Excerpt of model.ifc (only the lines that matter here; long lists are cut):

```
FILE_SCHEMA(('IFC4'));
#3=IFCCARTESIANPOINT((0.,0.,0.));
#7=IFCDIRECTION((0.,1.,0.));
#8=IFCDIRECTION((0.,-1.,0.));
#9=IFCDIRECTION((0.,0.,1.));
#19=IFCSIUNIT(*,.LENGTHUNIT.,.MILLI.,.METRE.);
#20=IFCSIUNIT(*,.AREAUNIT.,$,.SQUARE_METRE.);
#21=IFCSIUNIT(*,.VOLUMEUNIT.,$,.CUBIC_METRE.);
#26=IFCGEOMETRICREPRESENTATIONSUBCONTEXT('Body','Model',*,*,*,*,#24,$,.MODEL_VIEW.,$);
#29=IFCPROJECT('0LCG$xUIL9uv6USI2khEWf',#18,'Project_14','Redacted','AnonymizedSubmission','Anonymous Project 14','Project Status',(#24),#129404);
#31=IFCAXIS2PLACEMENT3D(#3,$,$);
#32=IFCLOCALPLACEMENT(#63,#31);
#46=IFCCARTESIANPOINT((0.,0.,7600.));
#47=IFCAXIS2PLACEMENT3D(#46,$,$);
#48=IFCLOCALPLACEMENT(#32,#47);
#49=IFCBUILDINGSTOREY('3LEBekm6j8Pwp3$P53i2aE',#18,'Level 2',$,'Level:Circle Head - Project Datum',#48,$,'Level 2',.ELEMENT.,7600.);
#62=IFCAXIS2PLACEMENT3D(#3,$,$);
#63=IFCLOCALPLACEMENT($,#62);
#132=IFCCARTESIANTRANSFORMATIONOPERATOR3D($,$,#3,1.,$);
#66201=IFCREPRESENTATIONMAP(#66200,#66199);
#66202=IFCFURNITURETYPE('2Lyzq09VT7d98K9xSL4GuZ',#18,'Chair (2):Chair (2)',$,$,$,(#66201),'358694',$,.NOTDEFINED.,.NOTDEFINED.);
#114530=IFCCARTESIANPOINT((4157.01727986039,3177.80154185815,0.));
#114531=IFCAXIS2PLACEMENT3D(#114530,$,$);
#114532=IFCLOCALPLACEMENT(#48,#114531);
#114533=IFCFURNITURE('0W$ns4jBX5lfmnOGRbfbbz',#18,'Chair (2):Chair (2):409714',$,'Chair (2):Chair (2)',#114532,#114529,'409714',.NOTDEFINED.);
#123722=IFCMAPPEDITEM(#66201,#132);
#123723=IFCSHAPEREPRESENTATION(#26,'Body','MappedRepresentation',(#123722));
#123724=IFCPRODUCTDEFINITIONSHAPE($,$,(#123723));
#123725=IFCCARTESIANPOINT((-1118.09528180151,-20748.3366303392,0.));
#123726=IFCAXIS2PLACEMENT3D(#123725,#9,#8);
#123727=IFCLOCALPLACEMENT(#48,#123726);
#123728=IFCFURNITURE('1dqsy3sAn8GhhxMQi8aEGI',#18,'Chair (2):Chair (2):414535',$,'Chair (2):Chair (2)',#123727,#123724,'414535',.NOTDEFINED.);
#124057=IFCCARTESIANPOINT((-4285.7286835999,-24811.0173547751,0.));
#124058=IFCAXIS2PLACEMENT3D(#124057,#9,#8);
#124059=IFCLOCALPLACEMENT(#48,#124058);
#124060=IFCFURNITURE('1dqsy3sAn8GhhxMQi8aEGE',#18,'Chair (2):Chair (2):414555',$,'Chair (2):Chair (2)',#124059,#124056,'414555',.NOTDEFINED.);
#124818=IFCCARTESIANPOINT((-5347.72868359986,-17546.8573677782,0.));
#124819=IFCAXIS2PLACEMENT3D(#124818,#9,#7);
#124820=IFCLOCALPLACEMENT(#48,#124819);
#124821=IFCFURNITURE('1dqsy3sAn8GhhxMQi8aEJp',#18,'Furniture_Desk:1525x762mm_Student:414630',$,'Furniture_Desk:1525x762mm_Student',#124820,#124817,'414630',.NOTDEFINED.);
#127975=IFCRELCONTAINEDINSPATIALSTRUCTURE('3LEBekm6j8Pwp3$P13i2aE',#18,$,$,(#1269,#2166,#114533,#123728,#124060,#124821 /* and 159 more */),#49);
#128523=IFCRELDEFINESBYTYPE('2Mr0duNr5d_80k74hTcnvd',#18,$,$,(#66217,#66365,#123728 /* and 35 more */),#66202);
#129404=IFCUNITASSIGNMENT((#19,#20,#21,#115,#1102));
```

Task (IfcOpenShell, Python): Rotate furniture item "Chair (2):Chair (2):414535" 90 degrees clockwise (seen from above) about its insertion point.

```python
import ifcopenshell
import ifcopenshell.api.geometry
import ifcopenshell.util.placement

model = ifcopenshell.open("model.ifc")

item = model.by_guid("1dqsy3sAn8GhhxMQi8aEGI")
matrix = ifcopenshell.util.placement.get_local_placement(item.ObjectPlacement)
matrix = matrix @ ifcopenshell.util.placement.rotation(-90, "Z")
ifcopenshell.api.geometry.edit_object_placement(model, product=item, matrix=matrix, is_si=False)

print(ifcopenshell.util.placement.get_local_placement(item.ObjectPlacement).round(3) + 0.0)

model.write("model_edited.ifc")
```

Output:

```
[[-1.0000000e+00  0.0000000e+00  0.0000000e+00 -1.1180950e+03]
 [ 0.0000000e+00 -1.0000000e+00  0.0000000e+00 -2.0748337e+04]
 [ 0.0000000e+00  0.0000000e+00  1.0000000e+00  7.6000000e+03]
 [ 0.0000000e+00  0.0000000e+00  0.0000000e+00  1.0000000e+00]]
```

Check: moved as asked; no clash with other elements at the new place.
